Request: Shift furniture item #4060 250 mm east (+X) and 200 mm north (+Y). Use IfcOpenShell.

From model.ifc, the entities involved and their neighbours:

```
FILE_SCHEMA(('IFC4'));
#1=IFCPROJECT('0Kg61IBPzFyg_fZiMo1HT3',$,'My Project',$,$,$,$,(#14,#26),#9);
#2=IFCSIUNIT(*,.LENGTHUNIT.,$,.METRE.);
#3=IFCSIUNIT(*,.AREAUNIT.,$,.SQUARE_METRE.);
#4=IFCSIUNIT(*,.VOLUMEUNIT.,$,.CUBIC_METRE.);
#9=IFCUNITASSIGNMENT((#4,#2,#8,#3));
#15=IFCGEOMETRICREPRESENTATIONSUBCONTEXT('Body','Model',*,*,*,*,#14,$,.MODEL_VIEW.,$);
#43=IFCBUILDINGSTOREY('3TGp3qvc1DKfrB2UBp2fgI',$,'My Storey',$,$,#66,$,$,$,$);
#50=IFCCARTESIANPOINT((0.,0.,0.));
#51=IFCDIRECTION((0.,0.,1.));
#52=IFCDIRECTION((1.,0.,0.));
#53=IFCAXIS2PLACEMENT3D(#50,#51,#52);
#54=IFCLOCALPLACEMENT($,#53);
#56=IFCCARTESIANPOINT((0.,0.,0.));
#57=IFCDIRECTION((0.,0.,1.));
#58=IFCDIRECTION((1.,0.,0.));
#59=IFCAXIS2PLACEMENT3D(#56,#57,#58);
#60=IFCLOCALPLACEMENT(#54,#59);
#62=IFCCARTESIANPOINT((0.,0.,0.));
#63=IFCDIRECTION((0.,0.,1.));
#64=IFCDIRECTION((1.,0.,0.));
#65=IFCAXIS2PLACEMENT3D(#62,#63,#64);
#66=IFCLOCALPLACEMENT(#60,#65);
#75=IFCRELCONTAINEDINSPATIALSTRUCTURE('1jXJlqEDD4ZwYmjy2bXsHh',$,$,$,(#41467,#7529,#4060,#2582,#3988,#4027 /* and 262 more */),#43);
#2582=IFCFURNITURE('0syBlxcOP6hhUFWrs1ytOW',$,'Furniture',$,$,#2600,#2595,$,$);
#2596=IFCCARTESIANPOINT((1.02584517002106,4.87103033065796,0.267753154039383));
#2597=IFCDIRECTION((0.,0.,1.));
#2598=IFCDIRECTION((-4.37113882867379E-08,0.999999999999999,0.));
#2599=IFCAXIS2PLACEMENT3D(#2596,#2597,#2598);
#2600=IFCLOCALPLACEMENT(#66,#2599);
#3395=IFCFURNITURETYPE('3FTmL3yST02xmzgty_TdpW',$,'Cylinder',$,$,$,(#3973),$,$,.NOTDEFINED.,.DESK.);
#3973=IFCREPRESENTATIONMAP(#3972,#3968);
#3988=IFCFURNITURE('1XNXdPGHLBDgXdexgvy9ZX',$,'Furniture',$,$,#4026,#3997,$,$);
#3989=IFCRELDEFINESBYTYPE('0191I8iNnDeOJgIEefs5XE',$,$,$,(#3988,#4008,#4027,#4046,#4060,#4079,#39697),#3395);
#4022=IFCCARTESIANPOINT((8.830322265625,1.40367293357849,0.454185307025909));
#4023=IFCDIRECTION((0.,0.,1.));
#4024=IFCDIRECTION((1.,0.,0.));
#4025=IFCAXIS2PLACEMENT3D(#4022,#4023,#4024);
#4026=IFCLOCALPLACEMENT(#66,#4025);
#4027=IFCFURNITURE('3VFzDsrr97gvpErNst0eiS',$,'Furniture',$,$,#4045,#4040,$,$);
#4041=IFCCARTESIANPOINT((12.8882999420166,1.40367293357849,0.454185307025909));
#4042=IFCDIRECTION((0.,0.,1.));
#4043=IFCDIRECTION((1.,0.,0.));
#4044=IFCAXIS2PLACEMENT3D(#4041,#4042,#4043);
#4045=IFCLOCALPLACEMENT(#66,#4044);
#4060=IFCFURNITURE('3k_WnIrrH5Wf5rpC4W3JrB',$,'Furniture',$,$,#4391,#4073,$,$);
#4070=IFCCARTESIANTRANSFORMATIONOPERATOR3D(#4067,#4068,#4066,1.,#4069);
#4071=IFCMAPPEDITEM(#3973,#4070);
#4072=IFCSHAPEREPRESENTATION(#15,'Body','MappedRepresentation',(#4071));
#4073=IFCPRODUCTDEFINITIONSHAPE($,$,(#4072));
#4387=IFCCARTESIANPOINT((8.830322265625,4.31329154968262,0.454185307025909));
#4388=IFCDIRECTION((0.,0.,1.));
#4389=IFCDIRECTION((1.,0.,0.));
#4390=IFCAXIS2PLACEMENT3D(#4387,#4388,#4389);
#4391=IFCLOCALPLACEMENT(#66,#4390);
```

```python
import ifcopenshell
import ifcopenshell.api.geometry
import ifcopenshell.util.placement
import ifcopenshell.util.unit

model = ifcopenshell.open("model.ifc")
unit_scale = ifcopenshell.util.unit.calculate_unit_scale(model)

item = model.by_guid("3k_WnIrrH5Wf5rpC4W3JrB")
matrix = ifcopenshell.util.placement.get_local_placement(item.ObjectPlacement)
matrix[0, 3] += 0.25 / unit_scale
matrix[1, 3] += 0.2 / unit_scale
ifcopenshell.api.geometry.edit_object_placement(model, product=item, matrix=matrix, is_si=False)

print(ifcopenshell.util.placement.get_local_placement(item.ObjectPlacement).round(3) + 0.0)

model.write("model_rev.ifc")
```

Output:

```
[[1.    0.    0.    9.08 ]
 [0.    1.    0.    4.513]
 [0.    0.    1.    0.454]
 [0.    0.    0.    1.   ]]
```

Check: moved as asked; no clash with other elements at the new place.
